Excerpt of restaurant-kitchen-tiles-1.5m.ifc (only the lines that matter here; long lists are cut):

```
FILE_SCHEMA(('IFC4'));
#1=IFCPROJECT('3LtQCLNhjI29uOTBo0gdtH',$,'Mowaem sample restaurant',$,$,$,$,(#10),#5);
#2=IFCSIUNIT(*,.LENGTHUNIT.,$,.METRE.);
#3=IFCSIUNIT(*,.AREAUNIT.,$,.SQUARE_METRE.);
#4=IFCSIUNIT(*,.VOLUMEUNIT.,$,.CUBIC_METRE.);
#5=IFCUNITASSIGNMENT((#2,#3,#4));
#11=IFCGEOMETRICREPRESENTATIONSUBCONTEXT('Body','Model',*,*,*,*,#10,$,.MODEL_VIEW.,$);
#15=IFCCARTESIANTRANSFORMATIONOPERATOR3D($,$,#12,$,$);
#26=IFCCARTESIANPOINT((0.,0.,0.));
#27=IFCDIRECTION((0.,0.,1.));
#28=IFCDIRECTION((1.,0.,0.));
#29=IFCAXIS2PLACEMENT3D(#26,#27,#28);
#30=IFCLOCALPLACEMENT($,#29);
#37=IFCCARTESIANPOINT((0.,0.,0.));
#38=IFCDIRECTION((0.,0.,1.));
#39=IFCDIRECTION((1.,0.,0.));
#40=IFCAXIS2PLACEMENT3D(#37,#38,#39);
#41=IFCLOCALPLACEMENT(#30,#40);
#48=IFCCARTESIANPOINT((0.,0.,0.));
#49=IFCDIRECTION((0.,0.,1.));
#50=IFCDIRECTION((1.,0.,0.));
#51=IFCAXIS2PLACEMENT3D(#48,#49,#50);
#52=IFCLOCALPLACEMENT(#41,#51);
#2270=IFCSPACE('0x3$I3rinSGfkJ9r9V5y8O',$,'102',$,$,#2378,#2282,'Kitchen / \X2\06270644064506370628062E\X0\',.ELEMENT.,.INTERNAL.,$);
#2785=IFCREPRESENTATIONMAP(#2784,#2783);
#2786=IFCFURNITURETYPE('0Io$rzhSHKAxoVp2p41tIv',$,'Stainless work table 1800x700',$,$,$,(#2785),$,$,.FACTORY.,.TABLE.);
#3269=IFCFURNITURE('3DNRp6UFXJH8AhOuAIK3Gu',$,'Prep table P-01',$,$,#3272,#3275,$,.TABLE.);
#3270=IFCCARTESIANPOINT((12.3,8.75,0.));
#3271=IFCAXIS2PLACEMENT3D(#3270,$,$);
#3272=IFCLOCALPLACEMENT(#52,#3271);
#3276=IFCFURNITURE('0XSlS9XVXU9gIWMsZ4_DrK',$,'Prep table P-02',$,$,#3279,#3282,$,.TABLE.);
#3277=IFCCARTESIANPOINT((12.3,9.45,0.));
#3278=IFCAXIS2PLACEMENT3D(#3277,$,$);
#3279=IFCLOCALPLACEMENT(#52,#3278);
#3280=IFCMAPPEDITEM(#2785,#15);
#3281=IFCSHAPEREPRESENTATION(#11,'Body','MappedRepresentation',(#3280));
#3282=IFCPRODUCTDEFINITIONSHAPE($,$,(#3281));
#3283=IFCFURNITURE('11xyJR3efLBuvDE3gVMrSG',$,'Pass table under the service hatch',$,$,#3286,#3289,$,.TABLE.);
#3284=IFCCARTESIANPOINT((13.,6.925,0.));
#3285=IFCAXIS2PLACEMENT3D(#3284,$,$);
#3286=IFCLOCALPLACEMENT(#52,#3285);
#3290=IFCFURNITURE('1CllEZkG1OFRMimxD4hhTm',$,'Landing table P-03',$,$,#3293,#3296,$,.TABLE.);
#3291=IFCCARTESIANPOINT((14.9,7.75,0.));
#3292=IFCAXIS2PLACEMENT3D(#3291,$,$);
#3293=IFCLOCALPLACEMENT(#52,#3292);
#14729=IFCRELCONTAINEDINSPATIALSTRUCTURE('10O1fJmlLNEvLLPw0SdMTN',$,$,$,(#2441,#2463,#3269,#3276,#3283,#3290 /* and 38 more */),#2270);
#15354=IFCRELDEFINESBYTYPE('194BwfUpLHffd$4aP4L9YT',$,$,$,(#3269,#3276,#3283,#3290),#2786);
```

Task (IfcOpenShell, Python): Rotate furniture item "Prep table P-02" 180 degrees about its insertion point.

```python
import ifcopenshell
import ifcopenshell.api.geometry
import ifcopenshell.util.placement

model = ifcopenshell.open("restaurant-kitchen-tiles-1.5m.ifc")

item = model.by_guid("0XSlS9XVXU9gIWMsZ4_DrK")
matrix = ifcopenshell.util.placement.get_local_placement(item.ObjectPlacement)
matrix = matrix @ ifcopenshell.util.placement.rotation(180, "Z")
ifcopenshell.api.geometry.edit_object_placement(model, product=item, matrix=matrix, is_si=False)

print(ifcopenshell.util.placement.get_local_placement(item.ObjectPlacement).round(3) + 0.0)

model.write("restaurant-kitchen-tiles-1.5m_updated.ifc")
```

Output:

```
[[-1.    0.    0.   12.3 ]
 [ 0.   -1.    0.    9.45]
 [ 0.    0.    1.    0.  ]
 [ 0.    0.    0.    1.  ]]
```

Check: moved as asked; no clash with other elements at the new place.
